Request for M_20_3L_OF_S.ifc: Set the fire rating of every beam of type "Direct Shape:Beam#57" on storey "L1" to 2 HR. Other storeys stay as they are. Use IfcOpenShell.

First a look at what the model holds.

```python
import ifcopenshell
import ifcopenshell.util.element

model = ifcopenshell.open("M_20_3L_OF_S.ifc")
print(model.schema)
storey = next(s for s in model.by_type("IfcBuildingStorey") if s.Name == "L1")
beams = [e for e in ifcopenshell.util.element.get_decomposition(storey) if e.is_a("IfcBeam")]
seen = {}
for e in beams:
    element_type = ifcopenshell.util.element.get_type(e)
    key = (element_type.Name if element_type != e and element_type else None, ifcopenshell.util.element.get_pset(e, "Pset_BeamCommon", "FireRating"))
    seen[key] = seen.get(key, 0) + 1
for (name, value), count in sorted(seen.items(), key=str):
    print(count, "x", name, "|", value)
```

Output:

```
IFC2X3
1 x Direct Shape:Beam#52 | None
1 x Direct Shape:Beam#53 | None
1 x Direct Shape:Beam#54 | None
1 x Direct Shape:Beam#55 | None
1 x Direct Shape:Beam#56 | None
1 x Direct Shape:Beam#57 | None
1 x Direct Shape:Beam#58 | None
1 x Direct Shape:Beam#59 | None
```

```python
import ifcopenshell
import ifcopenshell.api.pset
import ifcopenshell.util.element

model = ifcopenshell.open("M_20_3L_OF_S.ifc")

storey = next(s for s in model.by_type("IfcBuildingStorey") if s.Name == "L1")
beams = [e for e in ifcopenshell.util.element.get_decomposition(storey) if e.is_a("IfcBeam")]

count = 0
for e in beams:
    element_type = ifcopenshell.util.element.get_type(e)
    if element_type in (None, e) or element_type.Name != "Direct Shape:Beam#57":
        continue
    # add_pset returns the element's existing set when there is one.
    pset = ifcopenshell.api.pset.add_pset(model, product=e, name="Pset_BeamCommon")
    ifcopenshell.api.pset.edit_pset(model, pset=pset, properties={"FireRating": "2 HR"})
    count += 1

print(count, "beams updated")

model.write("M_20_3L_OF_S_v2.ifc")
```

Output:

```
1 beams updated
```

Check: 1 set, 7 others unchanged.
